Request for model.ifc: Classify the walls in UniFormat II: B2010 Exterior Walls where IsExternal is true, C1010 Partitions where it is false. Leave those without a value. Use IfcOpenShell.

First a look at what the model holds.

```python
import ifcopenshell
import ifcopenshell.util.element

model = ifcopenshell.open("model.ifc")
print(model.schema)
print("classifications:", [c.Name for c in model.by_type("IfcClassification")])
values = [ifcopenshell.util.element.get_pset(e, "Pset_WallCommon", "IsExternal") for e in model.by_type("IfcWall")]
for value in (True, False, None):
    print("IsExternal", value, values.count(value))
```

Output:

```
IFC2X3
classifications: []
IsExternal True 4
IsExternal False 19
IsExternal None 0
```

```python
import ifcopenshell
import ifcopenshell.api.classification
import ifcopenshell.util.element

model = ifcopenshell.open("model.ifc")

# IFC2X3 requires Source and Edition and has no link from the project to the system.
system = model.create_entity("IfcClassification", Source="ASTM", Edition="E1557", Name="UniFormat II")

walls = model.by_type("IfcWall")
external = {e: ifcopenshell.util.element.get_pset(e, "Pset_WallCommon", "IsExternal") for e in walls}
for flag, code, name in ((True, "B2010", "Exterior Walls"), (False, "C1010", "Partitions")):
    products = [e for e in walls if external[e] is flag]
    ifcopenshell.api.classification.add_reference(
        model, products=products, classification=system, identification=code, name=name
    )
    print(code, len(products))

model.write("model_edited.ifc")
```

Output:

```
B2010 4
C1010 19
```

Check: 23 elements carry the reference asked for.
